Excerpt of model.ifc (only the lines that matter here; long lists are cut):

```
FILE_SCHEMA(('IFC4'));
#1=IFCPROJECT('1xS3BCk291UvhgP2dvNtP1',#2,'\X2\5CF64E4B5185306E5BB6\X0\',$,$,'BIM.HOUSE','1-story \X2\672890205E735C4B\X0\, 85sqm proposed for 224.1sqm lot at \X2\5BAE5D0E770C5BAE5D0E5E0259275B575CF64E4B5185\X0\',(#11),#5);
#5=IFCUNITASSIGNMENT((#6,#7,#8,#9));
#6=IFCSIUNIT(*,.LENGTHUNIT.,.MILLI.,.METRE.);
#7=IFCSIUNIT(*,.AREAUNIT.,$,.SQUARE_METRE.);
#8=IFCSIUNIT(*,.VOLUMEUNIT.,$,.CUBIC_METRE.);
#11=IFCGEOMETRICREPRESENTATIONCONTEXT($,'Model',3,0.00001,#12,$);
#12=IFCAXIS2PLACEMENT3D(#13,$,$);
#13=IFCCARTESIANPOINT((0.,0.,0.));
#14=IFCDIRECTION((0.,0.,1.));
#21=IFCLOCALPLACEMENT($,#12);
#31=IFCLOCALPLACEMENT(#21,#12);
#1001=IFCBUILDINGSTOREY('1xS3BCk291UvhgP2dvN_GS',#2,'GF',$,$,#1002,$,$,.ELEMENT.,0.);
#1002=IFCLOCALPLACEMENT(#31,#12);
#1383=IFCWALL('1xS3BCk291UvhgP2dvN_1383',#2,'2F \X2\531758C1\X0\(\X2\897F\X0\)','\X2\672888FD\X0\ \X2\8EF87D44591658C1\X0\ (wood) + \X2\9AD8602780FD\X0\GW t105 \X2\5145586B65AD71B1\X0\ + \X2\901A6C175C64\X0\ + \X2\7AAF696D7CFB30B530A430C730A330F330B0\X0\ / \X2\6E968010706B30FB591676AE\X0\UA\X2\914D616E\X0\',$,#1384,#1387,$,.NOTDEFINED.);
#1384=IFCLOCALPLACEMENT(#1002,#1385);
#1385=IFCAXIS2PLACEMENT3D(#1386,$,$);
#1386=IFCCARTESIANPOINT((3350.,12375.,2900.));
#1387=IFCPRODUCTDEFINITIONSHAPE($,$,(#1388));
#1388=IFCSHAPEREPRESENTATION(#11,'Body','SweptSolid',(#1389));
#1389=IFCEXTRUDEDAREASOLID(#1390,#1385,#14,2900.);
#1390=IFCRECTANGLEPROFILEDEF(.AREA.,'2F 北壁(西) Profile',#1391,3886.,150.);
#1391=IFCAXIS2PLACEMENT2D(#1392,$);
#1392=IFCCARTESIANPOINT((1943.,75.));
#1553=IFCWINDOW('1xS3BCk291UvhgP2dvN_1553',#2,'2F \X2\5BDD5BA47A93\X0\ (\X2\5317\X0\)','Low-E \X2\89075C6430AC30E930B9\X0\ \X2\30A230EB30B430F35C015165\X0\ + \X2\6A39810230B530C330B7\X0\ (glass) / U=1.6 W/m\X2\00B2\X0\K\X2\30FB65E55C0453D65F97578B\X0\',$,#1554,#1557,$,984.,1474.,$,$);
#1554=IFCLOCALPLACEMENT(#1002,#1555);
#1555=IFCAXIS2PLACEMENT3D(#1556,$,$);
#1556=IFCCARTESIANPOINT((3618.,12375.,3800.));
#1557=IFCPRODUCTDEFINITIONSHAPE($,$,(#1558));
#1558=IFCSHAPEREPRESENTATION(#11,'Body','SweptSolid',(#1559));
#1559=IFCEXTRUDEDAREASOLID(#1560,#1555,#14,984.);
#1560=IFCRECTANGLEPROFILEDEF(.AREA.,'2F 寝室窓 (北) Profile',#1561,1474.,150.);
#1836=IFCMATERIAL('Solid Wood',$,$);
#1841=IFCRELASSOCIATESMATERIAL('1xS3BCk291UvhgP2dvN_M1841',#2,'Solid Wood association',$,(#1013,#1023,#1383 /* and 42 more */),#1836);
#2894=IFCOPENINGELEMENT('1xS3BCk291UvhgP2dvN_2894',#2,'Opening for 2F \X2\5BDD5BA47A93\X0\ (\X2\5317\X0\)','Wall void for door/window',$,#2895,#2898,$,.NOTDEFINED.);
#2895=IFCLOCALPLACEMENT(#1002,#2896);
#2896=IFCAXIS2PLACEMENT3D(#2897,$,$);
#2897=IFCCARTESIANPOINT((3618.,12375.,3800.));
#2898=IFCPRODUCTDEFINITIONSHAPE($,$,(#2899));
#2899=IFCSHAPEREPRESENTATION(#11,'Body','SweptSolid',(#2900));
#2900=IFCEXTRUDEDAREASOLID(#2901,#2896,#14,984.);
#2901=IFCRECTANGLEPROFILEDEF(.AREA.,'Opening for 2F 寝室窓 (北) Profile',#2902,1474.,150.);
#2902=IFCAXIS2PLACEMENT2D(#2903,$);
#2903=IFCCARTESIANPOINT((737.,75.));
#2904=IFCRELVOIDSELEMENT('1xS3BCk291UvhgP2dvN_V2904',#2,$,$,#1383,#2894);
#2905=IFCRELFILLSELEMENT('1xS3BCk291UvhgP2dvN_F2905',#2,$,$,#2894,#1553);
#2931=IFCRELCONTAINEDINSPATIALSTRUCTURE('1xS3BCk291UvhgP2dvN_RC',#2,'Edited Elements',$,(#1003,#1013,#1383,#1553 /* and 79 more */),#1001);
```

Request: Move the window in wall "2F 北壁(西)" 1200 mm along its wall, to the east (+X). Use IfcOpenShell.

```python
import ifcopenshell
import ifcopenshell.api.geometry
import ifcopenshell.util.placement
import ifcopenshell.util.unit

model = ifcopenshell.open("model.ifc")
unit_scale = ifcopenshell.util.unit.calculate_unit_scale(model)

window = model.by_guid("1xS3BCk291UvhgP2dvN_1553")
opening = window.FillsVoids[0].RelatingOpeningElement
wall = opening.VoidsElements[0].RelatingBuildingElement

wall_matrix = ifcopenshell.util.placement.get_local_placement(wall.ObjectPlacement)
shift = wall_matrix[:3, 0] * 1.2 / unit_scale
before = ifcopenshell.util.placement.get_local_placement(window.ObjectPlacement)[:3, 3].copy()

# The window is not placed relative to its opening, so move both.
for product in (opening, window):
    matrix = ifcopenshell.util.placement.get_local_placement(product.ObjectPlacement)
    matrix[:3, 3] += shift
    ifcopenshell.api.geometry.edit_object_placement(model, product=product, matrix=matrix, is_si=False)

after = ifcopenshell.util.placement.get_local_placement(window.ObjectPlacement)[:3, 3]
print("window moved by", (after - before).round(3) + 0.0)

model.write("model-out.ifc")
```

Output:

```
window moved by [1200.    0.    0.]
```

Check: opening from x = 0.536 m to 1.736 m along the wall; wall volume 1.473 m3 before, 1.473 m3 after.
